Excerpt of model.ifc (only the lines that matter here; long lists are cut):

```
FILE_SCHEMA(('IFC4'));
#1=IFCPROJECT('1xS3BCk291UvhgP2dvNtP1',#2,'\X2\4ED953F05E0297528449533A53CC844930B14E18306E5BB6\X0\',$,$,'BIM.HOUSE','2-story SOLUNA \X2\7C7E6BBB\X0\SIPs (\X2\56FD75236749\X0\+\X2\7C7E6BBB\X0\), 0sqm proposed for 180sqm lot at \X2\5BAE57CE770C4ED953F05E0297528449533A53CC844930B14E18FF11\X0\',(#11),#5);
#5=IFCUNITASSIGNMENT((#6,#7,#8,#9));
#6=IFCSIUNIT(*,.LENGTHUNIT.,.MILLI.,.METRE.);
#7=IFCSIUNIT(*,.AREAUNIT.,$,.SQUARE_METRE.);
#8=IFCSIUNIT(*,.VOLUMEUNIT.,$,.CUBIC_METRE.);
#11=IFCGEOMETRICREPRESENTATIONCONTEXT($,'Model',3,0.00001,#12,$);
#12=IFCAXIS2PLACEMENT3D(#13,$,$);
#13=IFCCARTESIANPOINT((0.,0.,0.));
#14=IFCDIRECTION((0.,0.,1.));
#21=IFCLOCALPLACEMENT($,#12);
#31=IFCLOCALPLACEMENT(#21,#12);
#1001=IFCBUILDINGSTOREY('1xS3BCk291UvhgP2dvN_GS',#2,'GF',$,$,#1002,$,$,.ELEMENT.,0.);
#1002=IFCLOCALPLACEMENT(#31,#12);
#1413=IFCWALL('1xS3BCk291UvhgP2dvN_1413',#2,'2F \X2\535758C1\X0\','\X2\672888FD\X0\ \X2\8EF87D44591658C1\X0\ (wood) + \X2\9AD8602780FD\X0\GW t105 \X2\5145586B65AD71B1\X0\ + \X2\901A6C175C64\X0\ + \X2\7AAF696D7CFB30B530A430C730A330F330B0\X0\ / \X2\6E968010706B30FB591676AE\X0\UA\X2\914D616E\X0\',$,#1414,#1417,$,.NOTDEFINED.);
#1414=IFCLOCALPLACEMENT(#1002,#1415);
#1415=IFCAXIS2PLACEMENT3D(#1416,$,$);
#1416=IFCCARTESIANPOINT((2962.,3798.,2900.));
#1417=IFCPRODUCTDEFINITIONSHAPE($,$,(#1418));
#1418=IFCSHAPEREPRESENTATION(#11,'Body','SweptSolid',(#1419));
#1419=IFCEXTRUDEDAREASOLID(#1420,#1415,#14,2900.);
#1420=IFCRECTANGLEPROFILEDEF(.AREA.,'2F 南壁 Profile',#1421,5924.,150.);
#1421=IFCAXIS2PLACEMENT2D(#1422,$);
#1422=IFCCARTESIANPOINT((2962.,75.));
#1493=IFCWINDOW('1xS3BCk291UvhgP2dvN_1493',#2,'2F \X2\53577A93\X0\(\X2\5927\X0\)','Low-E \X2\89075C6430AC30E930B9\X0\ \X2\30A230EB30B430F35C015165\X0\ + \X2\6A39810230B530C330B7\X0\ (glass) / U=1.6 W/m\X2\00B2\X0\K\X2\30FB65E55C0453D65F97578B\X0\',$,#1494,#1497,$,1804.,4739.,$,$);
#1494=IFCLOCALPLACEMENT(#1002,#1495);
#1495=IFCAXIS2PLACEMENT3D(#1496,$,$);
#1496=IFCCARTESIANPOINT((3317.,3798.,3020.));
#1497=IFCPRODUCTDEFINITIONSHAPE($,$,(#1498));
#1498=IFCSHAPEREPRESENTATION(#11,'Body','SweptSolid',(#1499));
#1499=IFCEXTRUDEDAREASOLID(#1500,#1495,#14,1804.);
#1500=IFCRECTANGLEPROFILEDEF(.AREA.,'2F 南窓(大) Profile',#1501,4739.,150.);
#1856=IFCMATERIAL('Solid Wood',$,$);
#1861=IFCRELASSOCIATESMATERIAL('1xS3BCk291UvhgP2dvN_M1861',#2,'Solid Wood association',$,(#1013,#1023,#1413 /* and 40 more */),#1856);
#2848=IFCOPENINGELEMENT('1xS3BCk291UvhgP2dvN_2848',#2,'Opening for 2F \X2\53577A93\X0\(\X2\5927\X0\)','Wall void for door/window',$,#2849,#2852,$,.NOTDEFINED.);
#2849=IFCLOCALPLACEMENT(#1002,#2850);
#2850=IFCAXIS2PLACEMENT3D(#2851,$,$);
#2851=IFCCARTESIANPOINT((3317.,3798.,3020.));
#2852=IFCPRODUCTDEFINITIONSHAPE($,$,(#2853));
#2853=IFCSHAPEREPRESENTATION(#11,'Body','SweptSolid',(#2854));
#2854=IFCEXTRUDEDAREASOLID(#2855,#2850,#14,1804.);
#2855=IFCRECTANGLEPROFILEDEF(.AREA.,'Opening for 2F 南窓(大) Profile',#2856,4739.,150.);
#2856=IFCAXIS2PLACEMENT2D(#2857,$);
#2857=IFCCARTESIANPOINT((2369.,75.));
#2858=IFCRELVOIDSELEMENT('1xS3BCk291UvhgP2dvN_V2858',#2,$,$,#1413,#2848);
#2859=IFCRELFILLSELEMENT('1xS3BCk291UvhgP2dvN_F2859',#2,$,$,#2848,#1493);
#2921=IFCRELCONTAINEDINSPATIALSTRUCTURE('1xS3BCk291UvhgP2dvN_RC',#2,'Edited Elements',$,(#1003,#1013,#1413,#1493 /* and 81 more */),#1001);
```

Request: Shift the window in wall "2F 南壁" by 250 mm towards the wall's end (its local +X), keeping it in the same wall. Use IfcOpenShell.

```python
import ifcopenshell
import ifcopenshell.api.geometry
import ifcopenshell.util.placement
import ifcopenshell.util.unit

model = ifcopenshell.open("model.ifc")
unit_scale = ifcopenshell.util.unit.calculate_unit_scale(model)

window = model.by_id(1493)
opening = window.FillsVoids[0].RelatingOpeningElement
wall = opening.VoidsElements[0].RelatingBuildingElement

wall_matrix = ifcopenshell.util.placement.get_local_placement(wall.ObjectPlacement)
shift = wall_matrix[:3, 0] * 0.25 / unit_scale
before = ifcopenshell.util.placement.get_local_placement(window.ObjectPlacement)[:3, 3].copy()

# The window is not placed relative to its opening, so move both.
for product in (opening, window):
    matrix = ifcopenshell.util.placement.get_local_placement(product.ObjectPlacement)
    matrix[:3, 3] += shift
    ifcopenshell.api.geometry.edit_object_placement(model, product=product, matrix=matrix, is_si=False)

after = ifcopenshell.util.placement.get_local_placement(window.ObjectPlacement)[:3, 3]
print("window moved by", (after - before).round(3) + 0.0)

model.write("model_rev.ifc")
```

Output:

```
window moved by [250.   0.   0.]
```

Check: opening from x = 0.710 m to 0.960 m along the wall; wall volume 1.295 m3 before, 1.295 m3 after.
